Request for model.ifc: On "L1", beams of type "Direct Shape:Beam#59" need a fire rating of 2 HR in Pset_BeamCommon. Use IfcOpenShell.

First a look at what the model holds.

```python
import ifcopenshell
import ifcopenshell.util.element

model = ifcopenshell.open("model.ifc")
print(model.schema)
storey = next(s for s in model.by_type("IfcBuildingStorey") if s.Name == "L1")
beams = [e for e in ifcopenshell.util.element.get_decomposition(storey) if e.is_a("IfcBeam")]
seen = {}
for e in beams:
    element_type = ifcopenshell.util.element.get_type(e)
    key = (element_type.Name if element_type != e and element_type else None, ifcopenshell.util.element.get_pset(e, "Pset_BeamCommon", "FireRating"))
    seen[key] = seen.get(key, 0) + 1
for (name, value), count in sorted(seen.items(), key=str):
    print(count, "x", name, "|", value)
```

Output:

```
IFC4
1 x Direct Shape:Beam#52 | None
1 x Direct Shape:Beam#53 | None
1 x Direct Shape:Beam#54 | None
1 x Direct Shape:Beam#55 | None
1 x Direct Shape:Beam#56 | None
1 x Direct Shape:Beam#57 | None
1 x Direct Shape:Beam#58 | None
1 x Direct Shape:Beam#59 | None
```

```python
import ifcopenshell
import ifcopenshell.api.pset
import ifcopenshell.util.element

model = ifcopenshell.open("model.ifc")

storey = next(s for s in model.by_type("IfcBuildingStorey") if s.Name == "L1")
beams = [e for e in ifcopenshell.util.element.get_decomposition(storey) if e.is_a("IfcBeam")]

count = 0
for e in beams:
    element_type = ifcopenshell.util.element.get_type(e)
    if element_type in (None, e) or element_type.Name != "Direct Shape:Beam#59":
        continue
    # add_pset returns the element's existing set when there is one.
    pset = ifcopenshell.api.pset.add_pset(model, product=e, name="Pset_BeamCommon")
    ifcopenshell.api.pset.edit_pset(model, pset=pset, properties={"FireRating": "2 HR"})
    count += 1

print(count, "beams updated")

model.write("model_v2.ifc")
```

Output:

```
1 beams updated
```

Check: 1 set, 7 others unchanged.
